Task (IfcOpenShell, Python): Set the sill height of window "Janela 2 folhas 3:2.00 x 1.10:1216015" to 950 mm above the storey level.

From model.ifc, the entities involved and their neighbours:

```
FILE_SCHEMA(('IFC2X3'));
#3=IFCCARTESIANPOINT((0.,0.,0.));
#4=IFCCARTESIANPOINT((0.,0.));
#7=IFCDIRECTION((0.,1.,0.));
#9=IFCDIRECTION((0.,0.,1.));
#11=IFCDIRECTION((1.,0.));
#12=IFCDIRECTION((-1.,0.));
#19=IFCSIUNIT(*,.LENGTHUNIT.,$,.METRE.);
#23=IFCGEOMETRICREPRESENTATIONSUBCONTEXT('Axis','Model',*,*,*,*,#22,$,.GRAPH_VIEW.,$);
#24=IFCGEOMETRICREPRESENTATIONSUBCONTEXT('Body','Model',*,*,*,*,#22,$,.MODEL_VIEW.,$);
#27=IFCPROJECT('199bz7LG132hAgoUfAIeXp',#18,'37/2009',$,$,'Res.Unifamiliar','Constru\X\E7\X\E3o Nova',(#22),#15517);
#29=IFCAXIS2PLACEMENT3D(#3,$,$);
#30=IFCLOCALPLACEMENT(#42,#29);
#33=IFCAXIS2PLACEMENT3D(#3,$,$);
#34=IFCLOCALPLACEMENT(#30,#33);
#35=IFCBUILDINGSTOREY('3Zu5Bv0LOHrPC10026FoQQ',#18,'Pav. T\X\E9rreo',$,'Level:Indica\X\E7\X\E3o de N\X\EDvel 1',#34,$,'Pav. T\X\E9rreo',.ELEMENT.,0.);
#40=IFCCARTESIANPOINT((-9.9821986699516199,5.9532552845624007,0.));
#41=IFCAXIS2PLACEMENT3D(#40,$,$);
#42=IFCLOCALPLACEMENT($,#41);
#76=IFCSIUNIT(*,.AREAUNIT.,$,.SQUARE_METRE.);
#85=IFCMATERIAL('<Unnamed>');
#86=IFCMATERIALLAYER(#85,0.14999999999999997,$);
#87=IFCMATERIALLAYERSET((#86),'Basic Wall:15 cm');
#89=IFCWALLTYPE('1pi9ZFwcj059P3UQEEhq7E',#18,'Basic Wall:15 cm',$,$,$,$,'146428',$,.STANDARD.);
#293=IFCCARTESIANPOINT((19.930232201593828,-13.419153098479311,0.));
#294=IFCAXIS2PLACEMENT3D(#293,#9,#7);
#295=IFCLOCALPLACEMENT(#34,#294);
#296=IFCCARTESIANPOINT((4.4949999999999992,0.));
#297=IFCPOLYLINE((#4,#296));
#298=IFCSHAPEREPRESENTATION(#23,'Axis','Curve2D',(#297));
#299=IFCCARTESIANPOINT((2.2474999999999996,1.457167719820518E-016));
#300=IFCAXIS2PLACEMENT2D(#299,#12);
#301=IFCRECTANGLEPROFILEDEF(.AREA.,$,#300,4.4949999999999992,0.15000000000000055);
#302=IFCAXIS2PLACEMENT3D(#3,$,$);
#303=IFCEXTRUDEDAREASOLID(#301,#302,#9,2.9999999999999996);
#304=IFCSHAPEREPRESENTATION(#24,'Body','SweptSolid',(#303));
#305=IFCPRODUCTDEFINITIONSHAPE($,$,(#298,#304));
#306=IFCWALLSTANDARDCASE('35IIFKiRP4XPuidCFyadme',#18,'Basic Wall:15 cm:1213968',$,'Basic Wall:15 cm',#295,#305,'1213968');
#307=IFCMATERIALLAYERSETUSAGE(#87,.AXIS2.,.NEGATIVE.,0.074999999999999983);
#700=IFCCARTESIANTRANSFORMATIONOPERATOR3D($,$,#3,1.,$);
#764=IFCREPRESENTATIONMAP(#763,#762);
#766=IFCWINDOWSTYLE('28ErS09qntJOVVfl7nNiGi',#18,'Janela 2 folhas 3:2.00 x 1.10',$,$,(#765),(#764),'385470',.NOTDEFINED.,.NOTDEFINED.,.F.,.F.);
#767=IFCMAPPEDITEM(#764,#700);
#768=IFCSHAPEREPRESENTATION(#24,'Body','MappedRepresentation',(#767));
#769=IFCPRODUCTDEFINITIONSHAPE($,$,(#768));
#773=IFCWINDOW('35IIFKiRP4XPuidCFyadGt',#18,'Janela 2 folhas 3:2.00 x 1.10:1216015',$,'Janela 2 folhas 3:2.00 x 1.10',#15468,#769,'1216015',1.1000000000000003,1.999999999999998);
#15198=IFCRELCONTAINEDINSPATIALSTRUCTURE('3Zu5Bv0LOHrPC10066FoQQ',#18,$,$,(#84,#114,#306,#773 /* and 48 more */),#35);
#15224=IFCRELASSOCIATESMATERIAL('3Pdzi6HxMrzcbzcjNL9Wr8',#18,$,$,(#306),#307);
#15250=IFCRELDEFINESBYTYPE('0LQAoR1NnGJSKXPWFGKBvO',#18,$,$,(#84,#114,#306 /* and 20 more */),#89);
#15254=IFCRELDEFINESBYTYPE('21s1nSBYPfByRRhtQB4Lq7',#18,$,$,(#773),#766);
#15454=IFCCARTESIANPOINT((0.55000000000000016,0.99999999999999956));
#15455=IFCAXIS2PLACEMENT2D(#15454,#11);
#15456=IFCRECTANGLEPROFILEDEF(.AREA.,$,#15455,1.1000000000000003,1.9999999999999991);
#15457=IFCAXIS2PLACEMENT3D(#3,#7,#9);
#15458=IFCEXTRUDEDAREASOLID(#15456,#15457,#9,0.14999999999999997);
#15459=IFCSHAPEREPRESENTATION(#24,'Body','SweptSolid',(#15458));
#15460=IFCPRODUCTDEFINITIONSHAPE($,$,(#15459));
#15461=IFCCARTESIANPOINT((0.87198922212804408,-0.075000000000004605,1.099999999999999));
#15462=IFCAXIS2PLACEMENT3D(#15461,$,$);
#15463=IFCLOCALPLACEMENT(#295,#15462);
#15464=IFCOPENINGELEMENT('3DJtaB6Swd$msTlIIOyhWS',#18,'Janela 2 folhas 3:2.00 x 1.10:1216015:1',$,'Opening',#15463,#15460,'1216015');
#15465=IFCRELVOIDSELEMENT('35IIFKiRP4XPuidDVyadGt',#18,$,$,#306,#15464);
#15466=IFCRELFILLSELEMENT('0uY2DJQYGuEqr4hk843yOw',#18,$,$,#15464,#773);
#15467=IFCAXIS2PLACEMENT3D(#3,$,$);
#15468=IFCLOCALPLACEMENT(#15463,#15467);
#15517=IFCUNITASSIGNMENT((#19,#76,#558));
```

```python
import numpy as np
import ifcopenshell
import ifcopenshell.api.geometry
import ifcopenshell.geom
import ifcopenshell.util.element
import ifcopenshell.util.placement
import ifcopenshell.util.shape
import ifcopenshell.util.unit

model = ifcopenshell.open("model.ifc")
unit_scale = ifcopenshell.util.unit.calculate_unit_scale(model)

window = model.by_guid("35IIFKiRP4XPuidCFyadGt")
opening = window.FillsVoids[0].RelatingOpeningElement
storey = ifcopenshell.util.element.get_container(window, ifc_class="IfcBuildingStorey")
level = ifcopenshell.util.placement.get_local_placement(storey.ObjectPlacement)[2, 3]

# The opening's origin need not be at the sill, so measure its lowest point.
shape = ifcopenshell.geom.create_shape(ifcopenshell.geom.settings(), opening)
bottom = ifcopenshell.util.shape.get_shape_bottom_elevation(shape, shape.geometry) / unit_scale
dz = level + 0.95 - bottom

shift = np.array([0.0, 0.0, dz])
# The window is placed relative to its opening, so it follows when the opening moves.
matrix = ifcopenshell.util.placement.get_local_placement(opening.ObjectPlacement)
matrix[:3, 3] += shift
ifcopenshell.api.geometry.edit_object_placement(
    model, product=opening, matrix=matrix, is_si=False, should_transform_children=True
)

print(f"moved by {dz * unit_scale:+.3f} m")

model.write("model-out.ifc")
```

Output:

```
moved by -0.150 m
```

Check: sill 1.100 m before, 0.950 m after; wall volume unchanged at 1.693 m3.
